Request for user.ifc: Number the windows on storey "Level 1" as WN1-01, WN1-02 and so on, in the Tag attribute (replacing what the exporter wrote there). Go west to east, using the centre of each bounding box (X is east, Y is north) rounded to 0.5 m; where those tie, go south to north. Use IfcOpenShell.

First a look at what the model holds.

```python
import ifcopenshell
import ifcopenshell.util.element
import ifcopenshell.util.placement

model = ifcopenshell.open("user.ifc")
print(model.schema)
storey = next(s for s in model.by_type("IfcBuildingStorey") if s.Name == "Level 1")
windows = [e for e in ifcopenshell.util.element.get_decomposition(storey) if e.is_a("IfcWindow")]
for e in sorted(windows, key=lambda e: e.id()):
    origin = ifcopenshell.util.placement.get_local_placement(e.ObjectPlacement)[:3, 3]
    print(e.id(), e.Tag, e.Name, origin.round(2) + 0.0, sep=" | ")
```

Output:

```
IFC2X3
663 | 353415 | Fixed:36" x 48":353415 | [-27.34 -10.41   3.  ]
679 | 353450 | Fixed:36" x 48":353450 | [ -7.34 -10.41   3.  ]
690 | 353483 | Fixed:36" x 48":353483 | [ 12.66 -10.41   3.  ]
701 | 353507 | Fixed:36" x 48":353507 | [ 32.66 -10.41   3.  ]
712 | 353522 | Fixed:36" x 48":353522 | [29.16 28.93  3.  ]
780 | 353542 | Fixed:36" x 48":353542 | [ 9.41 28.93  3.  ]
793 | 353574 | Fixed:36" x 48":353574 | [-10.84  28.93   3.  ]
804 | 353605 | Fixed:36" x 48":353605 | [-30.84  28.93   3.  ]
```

```python
import ifcopenshell
import ifcopenshell.geom
import ifcopenshell.util.element
import ifcopenshell.util.shape

model = ifcopenshell.open("user.ifc")
settings = ifcopenshell.geom.settings()
settings.set("use-world-coords", True)


def centre(element):
    shape = ifcopenshell.geom.create_shape(settings, element)
    return ifcopenshell.util.shape.get_bbox_centroid(shape.geometry)


storey = next(s for s in model.by_type("IfcBuildingStorey") if s.Name == "Level 1")
windows = [e for e in ifcopenshell.util.element.get_decomposition(storey) if e.is_a("IfcWindow")]

# Insertion points can sit at a corner or the storey origin, so sort by the geometry (in metres).
centres = {e: centre(e) for e in windows}
windows.sort(key=lambda e: (round(centres[e][0] / 0.5), centres[e][1]))

for i, e in enumerate(windows, start=1):
    number = f"WN1-{i:02d}"
    e.Tag = number
    print(e.id(), number)

model.write("user_updated.ifc")
```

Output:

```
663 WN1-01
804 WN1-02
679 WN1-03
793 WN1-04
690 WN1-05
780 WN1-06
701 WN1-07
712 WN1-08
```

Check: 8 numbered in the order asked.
